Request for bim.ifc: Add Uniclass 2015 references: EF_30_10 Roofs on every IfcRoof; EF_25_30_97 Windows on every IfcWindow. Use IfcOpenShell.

First a look at what the model holds.

```python
import ifcopenshell

model = ifcopenshell.open("bim.ifc")
print(model.schema)
print("classifications:", [c.Name for c in model.by_type("IfcClassification")])
for ifc_class in ("IfcDoor", "IfcRoof", "IfcStair", "IfcWall", "IfcWindow"):
    print(ifc_class, len(model.by_type(ifc_class)))
```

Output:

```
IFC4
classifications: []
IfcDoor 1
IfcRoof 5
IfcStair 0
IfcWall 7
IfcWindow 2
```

```python
import ifcopenshell
import ifcopenshell.api.classification

model = ifcopenshell.open("bim.ifc")

system = ifcopenshell.api.classification.add_classification(model, classification="Uniclass 2015")

codes = {
    "IfcRoof": ("EF_30_10", "Roofs"),
    "IfcWindow": ("EF_25_30_97", "Windows"),
}
for ifc_class, (code, name) in codes.items():
    products = model.by_type(ifc_class)
    ifcopenshell.api.classification.add_reference(
        model, products=products, classification=system, identification=code, name=name
    )
    print(code, len(products))

model.write("bim_rev.ifc")
```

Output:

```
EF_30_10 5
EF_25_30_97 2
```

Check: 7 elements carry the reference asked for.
